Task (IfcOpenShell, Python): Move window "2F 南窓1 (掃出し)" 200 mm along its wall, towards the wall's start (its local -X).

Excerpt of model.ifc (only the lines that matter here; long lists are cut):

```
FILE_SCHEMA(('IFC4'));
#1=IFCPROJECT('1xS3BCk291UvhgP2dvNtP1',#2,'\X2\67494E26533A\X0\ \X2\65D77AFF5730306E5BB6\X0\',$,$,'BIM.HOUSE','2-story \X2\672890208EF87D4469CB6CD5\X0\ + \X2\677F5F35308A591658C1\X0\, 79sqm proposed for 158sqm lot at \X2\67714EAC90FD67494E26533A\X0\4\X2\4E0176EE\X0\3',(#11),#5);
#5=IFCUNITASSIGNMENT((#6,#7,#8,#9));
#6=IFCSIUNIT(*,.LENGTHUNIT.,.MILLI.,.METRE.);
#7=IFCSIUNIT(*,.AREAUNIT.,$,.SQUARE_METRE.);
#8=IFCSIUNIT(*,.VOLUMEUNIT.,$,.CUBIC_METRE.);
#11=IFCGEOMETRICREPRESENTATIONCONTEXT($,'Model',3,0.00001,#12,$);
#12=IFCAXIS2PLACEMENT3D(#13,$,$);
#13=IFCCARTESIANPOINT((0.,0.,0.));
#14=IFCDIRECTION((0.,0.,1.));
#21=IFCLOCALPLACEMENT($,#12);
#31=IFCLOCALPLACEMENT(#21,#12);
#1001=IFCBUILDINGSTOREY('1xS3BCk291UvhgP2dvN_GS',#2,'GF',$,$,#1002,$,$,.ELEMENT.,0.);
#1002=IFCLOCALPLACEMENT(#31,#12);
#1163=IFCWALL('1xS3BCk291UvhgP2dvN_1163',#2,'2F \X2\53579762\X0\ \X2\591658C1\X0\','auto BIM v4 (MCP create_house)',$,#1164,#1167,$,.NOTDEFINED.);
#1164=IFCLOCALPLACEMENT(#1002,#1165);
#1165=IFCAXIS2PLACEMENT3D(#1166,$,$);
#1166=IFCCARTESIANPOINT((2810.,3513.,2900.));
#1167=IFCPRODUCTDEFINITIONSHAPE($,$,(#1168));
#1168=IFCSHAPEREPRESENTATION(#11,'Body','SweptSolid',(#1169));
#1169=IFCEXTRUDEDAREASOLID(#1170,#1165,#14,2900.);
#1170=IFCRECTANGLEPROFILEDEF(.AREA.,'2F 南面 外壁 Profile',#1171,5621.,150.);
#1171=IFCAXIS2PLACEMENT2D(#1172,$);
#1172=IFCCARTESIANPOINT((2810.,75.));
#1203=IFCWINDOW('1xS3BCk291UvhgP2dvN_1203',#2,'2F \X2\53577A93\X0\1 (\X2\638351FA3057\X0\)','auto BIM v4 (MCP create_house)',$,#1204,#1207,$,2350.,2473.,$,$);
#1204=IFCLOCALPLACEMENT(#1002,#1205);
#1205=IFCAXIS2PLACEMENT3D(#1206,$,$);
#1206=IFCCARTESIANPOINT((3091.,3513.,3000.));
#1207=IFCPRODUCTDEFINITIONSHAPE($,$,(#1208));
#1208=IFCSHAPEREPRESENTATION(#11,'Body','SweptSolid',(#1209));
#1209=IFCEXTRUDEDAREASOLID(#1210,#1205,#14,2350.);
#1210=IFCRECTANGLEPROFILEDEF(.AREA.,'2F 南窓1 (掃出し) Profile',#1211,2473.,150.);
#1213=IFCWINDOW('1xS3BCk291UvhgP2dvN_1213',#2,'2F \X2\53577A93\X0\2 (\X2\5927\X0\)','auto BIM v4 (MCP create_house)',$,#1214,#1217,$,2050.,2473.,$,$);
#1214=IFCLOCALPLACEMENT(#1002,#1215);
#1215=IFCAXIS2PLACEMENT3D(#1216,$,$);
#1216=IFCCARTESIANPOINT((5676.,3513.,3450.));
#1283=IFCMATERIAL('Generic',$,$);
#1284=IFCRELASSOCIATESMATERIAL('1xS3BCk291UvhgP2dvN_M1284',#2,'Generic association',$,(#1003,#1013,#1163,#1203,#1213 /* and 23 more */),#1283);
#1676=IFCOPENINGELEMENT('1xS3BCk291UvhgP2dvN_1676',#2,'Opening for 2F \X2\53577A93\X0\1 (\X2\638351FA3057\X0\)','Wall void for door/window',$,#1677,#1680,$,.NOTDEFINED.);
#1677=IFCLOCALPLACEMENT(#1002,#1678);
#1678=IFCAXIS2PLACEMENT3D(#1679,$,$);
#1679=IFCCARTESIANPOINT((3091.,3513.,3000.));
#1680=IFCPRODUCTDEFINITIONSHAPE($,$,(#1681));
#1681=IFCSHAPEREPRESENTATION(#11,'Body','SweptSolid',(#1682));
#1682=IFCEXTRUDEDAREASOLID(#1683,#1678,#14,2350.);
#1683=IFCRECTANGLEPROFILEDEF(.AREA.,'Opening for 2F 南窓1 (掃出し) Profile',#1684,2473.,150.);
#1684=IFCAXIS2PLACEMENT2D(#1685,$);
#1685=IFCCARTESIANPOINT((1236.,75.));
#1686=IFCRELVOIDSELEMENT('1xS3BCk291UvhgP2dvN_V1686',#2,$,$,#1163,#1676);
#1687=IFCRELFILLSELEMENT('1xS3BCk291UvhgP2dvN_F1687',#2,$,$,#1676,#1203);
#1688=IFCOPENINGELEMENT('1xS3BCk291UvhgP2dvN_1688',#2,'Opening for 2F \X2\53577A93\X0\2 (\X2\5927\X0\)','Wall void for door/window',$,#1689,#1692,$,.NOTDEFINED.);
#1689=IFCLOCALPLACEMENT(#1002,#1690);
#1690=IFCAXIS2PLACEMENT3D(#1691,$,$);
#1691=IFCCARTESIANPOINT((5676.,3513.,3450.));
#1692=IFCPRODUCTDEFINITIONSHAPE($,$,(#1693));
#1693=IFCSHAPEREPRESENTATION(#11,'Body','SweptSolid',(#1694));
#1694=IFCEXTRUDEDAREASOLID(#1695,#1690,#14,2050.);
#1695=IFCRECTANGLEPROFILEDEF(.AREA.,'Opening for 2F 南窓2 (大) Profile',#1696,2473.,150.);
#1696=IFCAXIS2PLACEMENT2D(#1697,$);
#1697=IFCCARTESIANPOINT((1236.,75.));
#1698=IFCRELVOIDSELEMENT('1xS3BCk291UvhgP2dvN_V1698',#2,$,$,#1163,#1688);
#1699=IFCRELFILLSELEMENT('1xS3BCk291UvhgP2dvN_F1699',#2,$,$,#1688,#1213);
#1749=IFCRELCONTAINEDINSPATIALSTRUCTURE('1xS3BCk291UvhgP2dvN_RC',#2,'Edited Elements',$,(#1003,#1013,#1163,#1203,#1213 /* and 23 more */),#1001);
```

```python
import ifcopenshell
import ifcopenshell.api.geometry
import ifcopenshell.util.placement
import ifcopenshell.util.unit

model = ifcopenshell.open("model.ifc")
unit_scale = ifcopenshell.util.unit.calculate_unit_scale(model)

window = model.by_guid("1xS3BCk291UvhgP2dvN_1203")
opening = window.FillsVoids[0].RelatingOpeningElement
wall = opening.VoidsElements[0].RelatingBuildingElement

wall_matrix = ifcopenshell.util.placement.get_local_placement(wall.ObjectPlacement)
shift = wall_matrix[:3, 0] * -0.2 / unit_scale
before = ifcopenshell.util.placement.get_local_placement(window.ObjectPlacement)[:3, 3].copy()

# The window is not placed relative to its opening, so move both.
for product in (opening, window):
    matrix = ifcopenshell.util.placement.get_local_placement(product.ObjectPlacement)
    matrix[:3, 3] += shift
    ifcopenshell.api.geometry.edit_object_placement(model, product=product, matrix=matrix, is_si=False)

after = ifcopenshell.util.placement.get_local_placement(window.ObjectPlacement)[:3, 3]
print("window moved by", (after - before).round(3) + 0.0)

model.write("model_edited.ifc")
```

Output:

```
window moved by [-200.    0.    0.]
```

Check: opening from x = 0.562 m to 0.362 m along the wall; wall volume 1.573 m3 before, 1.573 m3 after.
